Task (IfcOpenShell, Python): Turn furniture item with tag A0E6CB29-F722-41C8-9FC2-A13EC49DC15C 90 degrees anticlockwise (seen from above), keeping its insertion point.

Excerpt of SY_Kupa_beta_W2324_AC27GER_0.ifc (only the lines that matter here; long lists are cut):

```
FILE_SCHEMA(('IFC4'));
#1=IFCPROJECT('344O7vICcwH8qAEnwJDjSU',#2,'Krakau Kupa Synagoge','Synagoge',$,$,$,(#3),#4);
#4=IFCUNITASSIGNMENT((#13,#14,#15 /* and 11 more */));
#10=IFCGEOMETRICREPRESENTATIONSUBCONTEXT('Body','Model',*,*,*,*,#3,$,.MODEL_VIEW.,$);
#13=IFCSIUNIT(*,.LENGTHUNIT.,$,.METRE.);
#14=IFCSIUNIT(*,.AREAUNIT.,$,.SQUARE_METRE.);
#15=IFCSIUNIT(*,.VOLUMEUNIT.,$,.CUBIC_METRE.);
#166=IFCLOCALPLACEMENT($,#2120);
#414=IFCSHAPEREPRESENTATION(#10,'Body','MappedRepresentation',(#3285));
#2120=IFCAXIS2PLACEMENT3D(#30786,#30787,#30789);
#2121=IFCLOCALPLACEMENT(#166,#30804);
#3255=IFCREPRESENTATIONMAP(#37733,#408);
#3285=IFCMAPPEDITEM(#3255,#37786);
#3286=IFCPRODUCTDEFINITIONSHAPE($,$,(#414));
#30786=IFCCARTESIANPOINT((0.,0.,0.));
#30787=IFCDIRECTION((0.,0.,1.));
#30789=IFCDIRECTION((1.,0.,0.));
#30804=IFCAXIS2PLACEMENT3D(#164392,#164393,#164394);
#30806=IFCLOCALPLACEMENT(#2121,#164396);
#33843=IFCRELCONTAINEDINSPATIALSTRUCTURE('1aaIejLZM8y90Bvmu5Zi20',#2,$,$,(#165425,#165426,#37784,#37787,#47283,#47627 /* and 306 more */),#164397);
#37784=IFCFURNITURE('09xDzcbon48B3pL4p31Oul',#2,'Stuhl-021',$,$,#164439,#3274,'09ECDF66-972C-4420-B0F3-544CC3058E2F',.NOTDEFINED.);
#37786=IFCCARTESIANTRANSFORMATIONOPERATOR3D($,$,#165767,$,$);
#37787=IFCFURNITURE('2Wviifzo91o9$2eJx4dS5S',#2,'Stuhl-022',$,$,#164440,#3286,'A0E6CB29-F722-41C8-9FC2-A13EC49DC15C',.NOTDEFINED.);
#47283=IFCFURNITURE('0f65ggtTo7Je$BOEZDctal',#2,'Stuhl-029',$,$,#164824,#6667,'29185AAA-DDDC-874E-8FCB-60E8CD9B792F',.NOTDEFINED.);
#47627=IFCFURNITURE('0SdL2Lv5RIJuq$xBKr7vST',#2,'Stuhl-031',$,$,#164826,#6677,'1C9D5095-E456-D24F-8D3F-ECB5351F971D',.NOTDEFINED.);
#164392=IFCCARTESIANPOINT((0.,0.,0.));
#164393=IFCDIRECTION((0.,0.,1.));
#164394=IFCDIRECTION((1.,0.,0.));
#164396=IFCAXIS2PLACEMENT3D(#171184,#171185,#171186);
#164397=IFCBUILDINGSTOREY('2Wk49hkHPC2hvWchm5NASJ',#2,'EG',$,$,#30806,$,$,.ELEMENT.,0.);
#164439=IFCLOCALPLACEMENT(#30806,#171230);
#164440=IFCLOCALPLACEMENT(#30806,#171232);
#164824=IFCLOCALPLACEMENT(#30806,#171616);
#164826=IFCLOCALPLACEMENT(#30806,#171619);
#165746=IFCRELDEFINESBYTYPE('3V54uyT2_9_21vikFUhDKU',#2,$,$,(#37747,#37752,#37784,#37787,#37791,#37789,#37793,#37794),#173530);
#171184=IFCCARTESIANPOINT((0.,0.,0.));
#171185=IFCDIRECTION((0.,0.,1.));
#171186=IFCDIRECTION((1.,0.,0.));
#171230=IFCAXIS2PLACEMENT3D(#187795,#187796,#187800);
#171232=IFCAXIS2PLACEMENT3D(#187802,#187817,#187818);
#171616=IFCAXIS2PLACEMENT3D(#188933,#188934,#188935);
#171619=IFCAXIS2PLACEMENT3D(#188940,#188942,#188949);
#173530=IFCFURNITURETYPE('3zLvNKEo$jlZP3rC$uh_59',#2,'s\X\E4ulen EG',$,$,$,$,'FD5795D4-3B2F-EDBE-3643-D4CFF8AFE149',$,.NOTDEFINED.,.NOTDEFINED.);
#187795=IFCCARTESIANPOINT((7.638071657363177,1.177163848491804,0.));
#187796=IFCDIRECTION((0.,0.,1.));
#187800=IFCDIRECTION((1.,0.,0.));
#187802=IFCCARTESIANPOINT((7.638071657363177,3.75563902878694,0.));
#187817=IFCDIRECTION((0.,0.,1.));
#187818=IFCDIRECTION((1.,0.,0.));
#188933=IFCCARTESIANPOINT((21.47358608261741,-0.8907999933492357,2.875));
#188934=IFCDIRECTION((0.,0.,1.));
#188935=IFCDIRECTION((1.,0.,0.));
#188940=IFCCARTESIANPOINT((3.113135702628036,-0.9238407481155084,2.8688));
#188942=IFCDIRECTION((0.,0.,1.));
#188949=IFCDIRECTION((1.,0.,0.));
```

```python
import ifcopenshell
import ifcopenshell.api.geometry
import ifcopenshell.util.placement

model = ifcopenshell.open("SY_Kupa_beta_W2324_AC27GER_0.ifc")

item = model.by_guid("2Wviifzo91o9$2eJx4dS5S")
matrix = ifcopenshell.util.placement.get_local_placement(item.ObjectPlacement)
matrix = matrix @ ifcopenshell.util.placement.rotation(90, "Z")
ifcopenshell.api.geometry.edit_object_placement(model, product=item, matrix=matrix, is_si=False)

print(ifcopenshell.util.placement.get_local_placement(item.ObjectPlacement).round(3) + 0.0)

model.write("SY_Kupa_beta_W2324_AC27GER_0_v2.ifc")
```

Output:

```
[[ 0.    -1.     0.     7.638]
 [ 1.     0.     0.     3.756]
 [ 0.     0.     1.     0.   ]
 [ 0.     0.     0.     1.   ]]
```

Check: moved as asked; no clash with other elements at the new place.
